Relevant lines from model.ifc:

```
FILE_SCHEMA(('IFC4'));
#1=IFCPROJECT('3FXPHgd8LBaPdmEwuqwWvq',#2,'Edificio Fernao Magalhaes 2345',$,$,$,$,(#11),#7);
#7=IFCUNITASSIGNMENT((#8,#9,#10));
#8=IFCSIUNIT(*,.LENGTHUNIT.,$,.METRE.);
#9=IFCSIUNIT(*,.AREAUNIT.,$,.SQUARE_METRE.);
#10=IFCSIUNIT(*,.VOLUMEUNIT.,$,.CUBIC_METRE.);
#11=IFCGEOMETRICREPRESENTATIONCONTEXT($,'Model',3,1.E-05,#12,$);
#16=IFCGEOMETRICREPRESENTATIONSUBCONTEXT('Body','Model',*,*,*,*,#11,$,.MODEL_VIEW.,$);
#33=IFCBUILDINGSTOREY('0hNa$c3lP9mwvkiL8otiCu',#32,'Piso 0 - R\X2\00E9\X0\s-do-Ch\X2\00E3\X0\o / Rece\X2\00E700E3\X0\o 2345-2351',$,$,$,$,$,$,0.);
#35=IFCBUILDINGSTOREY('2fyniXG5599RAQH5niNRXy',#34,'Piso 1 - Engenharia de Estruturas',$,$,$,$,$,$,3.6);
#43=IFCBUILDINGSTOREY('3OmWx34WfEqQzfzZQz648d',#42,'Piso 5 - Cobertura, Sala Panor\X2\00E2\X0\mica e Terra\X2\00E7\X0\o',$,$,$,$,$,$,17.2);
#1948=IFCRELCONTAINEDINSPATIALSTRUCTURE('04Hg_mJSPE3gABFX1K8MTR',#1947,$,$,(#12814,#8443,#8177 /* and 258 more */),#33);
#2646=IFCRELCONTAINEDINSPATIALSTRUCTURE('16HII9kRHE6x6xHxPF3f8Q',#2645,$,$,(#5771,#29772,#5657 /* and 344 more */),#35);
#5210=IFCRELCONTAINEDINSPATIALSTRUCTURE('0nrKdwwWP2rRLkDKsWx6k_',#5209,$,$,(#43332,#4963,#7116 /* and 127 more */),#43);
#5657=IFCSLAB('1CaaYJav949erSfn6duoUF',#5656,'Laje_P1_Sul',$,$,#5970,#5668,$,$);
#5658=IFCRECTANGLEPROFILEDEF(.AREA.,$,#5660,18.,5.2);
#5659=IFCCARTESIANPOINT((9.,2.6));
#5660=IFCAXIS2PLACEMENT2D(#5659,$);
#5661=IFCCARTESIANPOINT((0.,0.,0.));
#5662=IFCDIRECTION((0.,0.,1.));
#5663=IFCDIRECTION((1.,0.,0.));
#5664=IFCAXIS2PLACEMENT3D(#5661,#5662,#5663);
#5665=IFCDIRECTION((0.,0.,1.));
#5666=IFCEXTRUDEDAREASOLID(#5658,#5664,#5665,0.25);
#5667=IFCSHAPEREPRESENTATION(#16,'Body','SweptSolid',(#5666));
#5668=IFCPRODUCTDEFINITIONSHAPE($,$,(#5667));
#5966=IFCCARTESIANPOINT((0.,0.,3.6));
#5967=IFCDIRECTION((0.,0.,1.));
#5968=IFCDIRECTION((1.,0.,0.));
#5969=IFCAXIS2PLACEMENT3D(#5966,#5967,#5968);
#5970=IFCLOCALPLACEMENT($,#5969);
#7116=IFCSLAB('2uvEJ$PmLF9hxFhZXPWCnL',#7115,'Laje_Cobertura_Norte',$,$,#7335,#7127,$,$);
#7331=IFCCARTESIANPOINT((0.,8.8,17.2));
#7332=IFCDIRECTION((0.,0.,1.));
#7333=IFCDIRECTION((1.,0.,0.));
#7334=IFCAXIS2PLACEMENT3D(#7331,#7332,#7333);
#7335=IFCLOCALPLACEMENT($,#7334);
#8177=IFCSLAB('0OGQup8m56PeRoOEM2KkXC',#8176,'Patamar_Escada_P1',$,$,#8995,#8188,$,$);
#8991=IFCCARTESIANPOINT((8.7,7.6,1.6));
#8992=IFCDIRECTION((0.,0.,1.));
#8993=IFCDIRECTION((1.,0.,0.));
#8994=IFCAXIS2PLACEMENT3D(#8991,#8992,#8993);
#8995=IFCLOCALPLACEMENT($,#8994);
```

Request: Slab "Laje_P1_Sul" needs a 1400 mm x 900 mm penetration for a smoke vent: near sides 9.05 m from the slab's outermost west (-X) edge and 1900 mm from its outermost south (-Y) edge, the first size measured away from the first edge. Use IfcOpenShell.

```python
import numpy as np
import ifcopenshell
import ifcopenshell.api.feature
import ifcopenshell.api.geometry
import ifcopenshell.api.root
import ifcopenshell.geom
import ifcopenshell.util.placement
import ifcopenshell.util.representation
import ifcopenshell.util.shape
import ifcopenshell.util.unit

model = ifcopenshell.open("model.ifc")
unit_scale = ifcopenshell.util.unit.calculate_unit_scale(model)
settings = ifcopenshell.geom.settings()


def volume(element):
    """Net volume in cubic metres, openings subtracted."""
    shape = ifcopenshell.geom.create_shape(settings, element)
    return ifcopenshell.util.shape.get_volume(shape.geometry)


slab = model.by_guid("1CaaYJav949erSfn6duoUF")
before = volume(slab)

# Extent in the slab's own axes, in metres. The edges named are its -X and -Y sides.
slab_shape = ifcopenshell.geom.create_shape(settings, slab)
vertices = ifcopenshell.util.shape.get_vertices(slab_shape.geometry)
x_min, y_min, bottom = vertices.min(axis=0)
top = vertices[:, 2].max()

opening = ifcopenshell.api.root.create_entity(model, ifc_class="IfcOpeningElement", name="Smoke vent opening", predefined_type="OPENING")
context = ifcopenshell.util.representation.get_context(model, "Model", "Body", "MODEL_VIEW")
width, depth = 1.4, 0.9
outline = [(0.0, 0.0), (width, 0.0), (width, depth), (0.0, depth), (0.0, 0.0)]
# Overshoot both faces by 50 mm so the cut is clean.
shape = ifcopenshell.api.geometry.add_slab_representation(
    model, context=context, depth=top - bottom + 0.1, polyline=outline
)
ifcopenshell.api.geometry.assign_representation(model, product=opening, representation=shape)

matrix = ifcopenshell.util.placement.get_local_placement(slab.ObjectPlacement)
matrix[:, 3] = matrix @ np.append(np.array([x_min + 9.05, y_min + 1.9, bottom - 0.05]) / unit_scale, 1.0)
ifcopenshell.api.geometry.edit_object_placement(model, product=opening, matrix=matrix, is_si=False)
ifcopenshell.api.feature.add_feature(model, feature=opening, element=slab)

after = volume(slab)

print(f"slab volume {before:.3f} -> {after:.3f} m3")

model.write("model-out.ifc")
```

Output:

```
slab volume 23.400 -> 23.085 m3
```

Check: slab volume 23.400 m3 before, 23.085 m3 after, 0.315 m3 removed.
